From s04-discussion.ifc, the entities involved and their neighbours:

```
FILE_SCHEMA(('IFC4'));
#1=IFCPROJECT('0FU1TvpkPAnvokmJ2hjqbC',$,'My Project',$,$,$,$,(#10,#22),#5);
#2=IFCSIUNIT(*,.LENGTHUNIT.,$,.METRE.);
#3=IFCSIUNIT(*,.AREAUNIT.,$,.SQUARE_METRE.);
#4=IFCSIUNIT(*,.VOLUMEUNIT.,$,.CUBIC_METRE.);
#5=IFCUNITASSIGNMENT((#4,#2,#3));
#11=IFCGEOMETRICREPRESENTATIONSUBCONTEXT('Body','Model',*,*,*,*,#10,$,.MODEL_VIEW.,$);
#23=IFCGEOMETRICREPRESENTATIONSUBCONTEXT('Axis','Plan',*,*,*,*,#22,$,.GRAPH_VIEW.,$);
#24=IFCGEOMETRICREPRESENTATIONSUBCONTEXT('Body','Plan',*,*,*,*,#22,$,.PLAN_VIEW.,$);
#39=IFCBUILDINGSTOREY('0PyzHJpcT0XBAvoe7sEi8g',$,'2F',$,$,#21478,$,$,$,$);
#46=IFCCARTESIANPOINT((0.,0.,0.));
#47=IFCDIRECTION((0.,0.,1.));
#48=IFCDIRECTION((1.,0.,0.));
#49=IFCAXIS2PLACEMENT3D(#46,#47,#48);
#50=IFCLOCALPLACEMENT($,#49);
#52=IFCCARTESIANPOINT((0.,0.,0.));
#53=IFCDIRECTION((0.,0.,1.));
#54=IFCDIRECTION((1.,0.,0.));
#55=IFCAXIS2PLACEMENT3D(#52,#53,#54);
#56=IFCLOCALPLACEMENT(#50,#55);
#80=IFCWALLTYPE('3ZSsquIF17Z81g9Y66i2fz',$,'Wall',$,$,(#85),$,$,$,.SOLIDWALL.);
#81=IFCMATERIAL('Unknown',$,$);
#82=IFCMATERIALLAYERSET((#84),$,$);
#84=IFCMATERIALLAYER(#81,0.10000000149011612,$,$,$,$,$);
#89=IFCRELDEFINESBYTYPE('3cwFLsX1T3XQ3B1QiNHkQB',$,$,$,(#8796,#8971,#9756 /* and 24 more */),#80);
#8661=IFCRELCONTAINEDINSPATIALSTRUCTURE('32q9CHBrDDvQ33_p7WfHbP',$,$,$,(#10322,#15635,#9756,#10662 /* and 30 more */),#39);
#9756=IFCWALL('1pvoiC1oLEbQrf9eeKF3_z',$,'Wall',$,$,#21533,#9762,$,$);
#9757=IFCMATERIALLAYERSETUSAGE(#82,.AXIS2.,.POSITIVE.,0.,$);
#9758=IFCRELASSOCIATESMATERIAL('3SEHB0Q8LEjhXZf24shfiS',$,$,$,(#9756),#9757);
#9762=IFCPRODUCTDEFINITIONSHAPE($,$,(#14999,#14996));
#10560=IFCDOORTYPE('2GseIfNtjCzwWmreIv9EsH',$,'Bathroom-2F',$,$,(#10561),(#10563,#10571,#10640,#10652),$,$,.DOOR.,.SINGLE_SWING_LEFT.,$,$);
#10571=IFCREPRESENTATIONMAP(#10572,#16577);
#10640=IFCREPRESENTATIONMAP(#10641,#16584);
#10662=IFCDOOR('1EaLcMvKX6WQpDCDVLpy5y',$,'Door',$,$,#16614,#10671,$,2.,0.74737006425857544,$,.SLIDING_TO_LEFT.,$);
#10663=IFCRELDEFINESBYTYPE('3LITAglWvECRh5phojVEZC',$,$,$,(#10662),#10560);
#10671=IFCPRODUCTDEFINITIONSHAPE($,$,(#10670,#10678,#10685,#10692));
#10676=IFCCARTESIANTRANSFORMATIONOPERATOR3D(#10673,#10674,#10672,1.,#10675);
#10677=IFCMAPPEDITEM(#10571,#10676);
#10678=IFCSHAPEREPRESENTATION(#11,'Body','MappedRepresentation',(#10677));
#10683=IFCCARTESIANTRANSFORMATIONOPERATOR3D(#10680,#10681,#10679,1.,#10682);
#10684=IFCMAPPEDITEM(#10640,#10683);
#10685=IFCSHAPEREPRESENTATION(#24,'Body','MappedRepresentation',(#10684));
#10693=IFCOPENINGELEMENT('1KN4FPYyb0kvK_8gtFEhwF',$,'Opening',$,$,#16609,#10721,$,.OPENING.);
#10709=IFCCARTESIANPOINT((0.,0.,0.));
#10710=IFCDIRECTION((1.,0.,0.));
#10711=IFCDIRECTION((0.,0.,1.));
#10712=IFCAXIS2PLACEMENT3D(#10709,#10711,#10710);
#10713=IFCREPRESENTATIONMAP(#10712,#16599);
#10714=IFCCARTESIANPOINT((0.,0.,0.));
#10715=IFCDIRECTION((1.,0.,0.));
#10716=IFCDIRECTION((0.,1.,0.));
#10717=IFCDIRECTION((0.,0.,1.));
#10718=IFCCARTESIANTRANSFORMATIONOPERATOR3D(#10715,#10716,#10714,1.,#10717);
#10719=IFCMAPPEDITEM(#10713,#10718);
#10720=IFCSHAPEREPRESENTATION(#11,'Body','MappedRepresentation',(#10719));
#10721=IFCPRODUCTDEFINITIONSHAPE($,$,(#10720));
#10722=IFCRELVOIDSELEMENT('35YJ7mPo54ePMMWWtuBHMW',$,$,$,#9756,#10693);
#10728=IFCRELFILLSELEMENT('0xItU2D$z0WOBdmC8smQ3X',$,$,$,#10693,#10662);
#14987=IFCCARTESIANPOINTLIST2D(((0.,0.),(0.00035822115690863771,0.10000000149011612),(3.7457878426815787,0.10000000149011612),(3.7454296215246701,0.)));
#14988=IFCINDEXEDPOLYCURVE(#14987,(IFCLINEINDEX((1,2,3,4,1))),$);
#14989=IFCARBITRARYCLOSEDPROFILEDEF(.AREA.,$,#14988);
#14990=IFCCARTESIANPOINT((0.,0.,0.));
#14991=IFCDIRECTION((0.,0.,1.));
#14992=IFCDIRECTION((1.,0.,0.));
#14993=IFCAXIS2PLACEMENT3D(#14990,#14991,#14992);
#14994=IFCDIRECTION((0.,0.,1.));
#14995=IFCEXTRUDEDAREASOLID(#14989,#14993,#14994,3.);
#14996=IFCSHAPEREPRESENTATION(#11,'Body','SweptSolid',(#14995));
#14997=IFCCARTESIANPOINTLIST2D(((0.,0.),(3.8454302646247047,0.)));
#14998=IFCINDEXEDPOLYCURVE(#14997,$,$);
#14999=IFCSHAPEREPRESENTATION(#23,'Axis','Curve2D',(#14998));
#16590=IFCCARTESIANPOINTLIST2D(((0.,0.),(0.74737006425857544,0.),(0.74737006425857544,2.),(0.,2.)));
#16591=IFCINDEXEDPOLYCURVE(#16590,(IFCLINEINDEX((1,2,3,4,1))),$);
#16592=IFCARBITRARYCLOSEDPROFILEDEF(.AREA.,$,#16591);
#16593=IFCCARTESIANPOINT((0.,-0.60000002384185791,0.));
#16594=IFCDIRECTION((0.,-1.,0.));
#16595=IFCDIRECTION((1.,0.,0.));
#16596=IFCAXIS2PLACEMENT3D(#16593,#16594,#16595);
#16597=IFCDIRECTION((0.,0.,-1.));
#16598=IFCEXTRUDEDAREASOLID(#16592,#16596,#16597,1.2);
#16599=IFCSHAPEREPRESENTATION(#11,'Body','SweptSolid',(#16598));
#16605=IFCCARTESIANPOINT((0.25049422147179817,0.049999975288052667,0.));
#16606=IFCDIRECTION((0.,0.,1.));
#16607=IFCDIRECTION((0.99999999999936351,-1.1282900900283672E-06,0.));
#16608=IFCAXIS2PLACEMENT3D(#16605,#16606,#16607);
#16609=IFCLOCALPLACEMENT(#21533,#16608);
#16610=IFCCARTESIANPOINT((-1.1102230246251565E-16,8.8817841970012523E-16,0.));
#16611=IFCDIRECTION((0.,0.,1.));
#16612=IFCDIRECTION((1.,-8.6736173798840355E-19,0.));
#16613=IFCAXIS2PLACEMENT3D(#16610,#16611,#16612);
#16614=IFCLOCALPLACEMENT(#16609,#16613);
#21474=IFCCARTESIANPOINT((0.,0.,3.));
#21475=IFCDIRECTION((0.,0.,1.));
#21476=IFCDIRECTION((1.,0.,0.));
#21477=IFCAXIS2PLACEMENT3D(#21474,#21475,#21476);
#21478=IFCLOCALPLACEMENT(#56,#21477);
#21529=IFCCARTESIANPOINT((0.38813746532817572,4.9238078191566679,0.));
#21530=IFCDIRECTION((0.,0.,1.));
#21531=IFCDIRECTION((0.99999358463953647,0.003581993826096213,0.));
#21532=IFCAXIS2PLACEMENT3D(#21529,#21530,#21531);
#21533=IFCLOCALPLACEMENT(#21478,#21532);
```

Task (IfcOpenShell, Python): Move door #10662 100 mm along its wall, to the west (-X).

```python
import ifcopenshell
import ifcopenshell.api.geometry
import ifcopenshell.util.placement
import ifcopenshell.util.unit

model = ifcopenshell.open("s04-discussion.ifc")
unit_scale = ifcopenshell.util.unit.calculate_unit_scale(model)

door = model.by_guid("1EaLcMvKX6WQpDCDVLpy5y")
opening = door.FillsVoids[0].RelatingOpeningElement
wall = opening.VoidsElements[0].RelatingBuildingElement

wall_matrix = ifcopenshell.util.placement.get_local_placement(wall.ObjectPlacement)
shift = wall_matrix[:3, 0] * -0.1 / unit_scale
before = ifcopenshell.util.placement.get_local_placement(door.ObjectPlacement)[:3, 3].copy()

# The door is placed relative to its opening, so it follows when the opening moves.
matrix = ifcopenshell.util.placement.get_local_placement(opening.ObjectPlacement)
matrix[:3, 3] += shift
ifcopenshell.api.geometry.edit_object_placement(
    model, product=opening, matrix=matrix, is_si=False, should_transform_children=True
)

after = ifcopenshell.util.placement.get_local_placement(door.ObjectPlacement)[:3, 3]
print("door moved by", (after - before).round(3) + 0.0)

model.write("s04-discussion-out.ifc")
```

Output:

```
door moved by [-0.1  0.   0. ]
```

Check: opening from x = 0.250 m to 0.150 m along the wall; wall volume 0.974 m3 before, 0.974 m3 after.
